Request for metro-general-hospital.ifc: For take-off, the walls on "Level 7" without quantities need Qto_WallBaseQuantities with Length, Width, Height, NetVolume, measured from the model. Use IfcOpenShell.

First a look at what the model holds.

```python
import ifcopenshell
import ifcopenshell.util.element
import ifcopenshell.util.unit

model = ifcopenshell.open("metro-general-hospital.ifc")
print(model.schema)
for unit_type in ("LENGTHUNIT", "AREAUNIT", "VOLUMEUNIT"):
    print(unit_type, ifcopenshell.util.unit.calculate_unit_scale(model, unit_type))
storey = next(s for s in model.by_type("IfcBuildingStorey") if s.Name == "Level 7")
walls = [e for e in ifcopenshell.util.element.get_decomposition(storey) if e.is_a("IfcWall")]
for e in sorted(walls, key=lambda e: e.id()):
    print(e.id(), e.is_a(), e.Name, list(ifcopenshell.util.element.get_psets(e, qtos_only=True)), sep=" | ")
```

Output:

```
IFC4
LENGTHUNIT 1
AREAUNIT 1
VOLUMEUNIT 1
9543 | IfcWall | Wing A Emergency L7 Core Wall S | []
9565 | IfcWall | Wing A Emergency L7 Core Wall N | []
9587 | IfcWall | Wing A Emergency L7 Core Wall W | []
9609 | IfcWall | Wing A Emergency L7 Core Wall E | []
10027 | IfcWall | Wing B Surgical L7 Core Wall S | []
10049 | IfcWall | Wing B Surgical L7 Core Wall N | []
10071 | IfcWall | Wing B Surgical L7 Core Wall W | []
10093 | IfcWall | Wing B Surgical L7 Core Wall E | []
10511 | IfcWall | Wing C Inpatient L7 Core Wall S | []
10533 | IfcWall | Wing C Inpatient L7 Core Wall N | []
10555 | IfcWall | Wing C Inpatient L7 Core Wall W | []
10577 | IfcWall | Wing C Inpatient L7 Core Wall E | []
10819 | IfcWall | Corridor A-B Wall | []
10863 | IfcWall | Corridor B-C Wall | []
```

```python
import ifcopenshell
import ifcopenshell.api.pset
import ifcopenshell.geom
import ifcopenshell.util.element
import ifcopenshell.util.shape
import ifcopenshell.util.unit

model = ifcopenshell.open("metro-general-hospital.ifc")
unit_scale = ifcopenshell.util.unit.calculate_unit_scale(model)
volume_scale = ifcopenshell.util.unit.calculate_unit_scale(model, "VOLUMEUNIT")
settings = ifcopenshell.geom.settings()

storey = next(s for s in model.by_type("IfcBuildingStorey") if s.Name == "Level 7")
walls = [e for e in ifcopenshell.util.element.get_decomposition(storey) if e.is_a("IfcWall")]

for e in sorted(walls, key=lambda e: e.id()):
    if ifcopenshell.util.element.get_psets(e, qtos_only=True, should_inherit=False):
        continue
    # Geometry comes back in metres, in the element's own axes.
    shape = ifcopenshell.geom.create_shape(settings, e)
    values = {
        "Length": ifcopenshell.util.shape.get_x(shape.geometry) / unit_scale,
        "Width": ifcopenshell.util.shape.get_y(shape.geometry) / unit_scale,
        "Height": ifcopenshell.util.shape.get_z(shape.geometry) / unit_scale,
        "NetVolume": ifcopenshell.util.shape.get_volume(shape.geometry) / volume_scale,
    }
    qto = ifcopenshell.api.pset.add_qto(model, product=e, name="Qto_WallBaseQuantities")
    ifcopenshell.api.pset.edit_qto(model, qto=qto, properties=values)
    print(e.id(), {k: round(v, 3) for k, v in values.items()})

model.write("metro-general-hospital_updated.ifc")
```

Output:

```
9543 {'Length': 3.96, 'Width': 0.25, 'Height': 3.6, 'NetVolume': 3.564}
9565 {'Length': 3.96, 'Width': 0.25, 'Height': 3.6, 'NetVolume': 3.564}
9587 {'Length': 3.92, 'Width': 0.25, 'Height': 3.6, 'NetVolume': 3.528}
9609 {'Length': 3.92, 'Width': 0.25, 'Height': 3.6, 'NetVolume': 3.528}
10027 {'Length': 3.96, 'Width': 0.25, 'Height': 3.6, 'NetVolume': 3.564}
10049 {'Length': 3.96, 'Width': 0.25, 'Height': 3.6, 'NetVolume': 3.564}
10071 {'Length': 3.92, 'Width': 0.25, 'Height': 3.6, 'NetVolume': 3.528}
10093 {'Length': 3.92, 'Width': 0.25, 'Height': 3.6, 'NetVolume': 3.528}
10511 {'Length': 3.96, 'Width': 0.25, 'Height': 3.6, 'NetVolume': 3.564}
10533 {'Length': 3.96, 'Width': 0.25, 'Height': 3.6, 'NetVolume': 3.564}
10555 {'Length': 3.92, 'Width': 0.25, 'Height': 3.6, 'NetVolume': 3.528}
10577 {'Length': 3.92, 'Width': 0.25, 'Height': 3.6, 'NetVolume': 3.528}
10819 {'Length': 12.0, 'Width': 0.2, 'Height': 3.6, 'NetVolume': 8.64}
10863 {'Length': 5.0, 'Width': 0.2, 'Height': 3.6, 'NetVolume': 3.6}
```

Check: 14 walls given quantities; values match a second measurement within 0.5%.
